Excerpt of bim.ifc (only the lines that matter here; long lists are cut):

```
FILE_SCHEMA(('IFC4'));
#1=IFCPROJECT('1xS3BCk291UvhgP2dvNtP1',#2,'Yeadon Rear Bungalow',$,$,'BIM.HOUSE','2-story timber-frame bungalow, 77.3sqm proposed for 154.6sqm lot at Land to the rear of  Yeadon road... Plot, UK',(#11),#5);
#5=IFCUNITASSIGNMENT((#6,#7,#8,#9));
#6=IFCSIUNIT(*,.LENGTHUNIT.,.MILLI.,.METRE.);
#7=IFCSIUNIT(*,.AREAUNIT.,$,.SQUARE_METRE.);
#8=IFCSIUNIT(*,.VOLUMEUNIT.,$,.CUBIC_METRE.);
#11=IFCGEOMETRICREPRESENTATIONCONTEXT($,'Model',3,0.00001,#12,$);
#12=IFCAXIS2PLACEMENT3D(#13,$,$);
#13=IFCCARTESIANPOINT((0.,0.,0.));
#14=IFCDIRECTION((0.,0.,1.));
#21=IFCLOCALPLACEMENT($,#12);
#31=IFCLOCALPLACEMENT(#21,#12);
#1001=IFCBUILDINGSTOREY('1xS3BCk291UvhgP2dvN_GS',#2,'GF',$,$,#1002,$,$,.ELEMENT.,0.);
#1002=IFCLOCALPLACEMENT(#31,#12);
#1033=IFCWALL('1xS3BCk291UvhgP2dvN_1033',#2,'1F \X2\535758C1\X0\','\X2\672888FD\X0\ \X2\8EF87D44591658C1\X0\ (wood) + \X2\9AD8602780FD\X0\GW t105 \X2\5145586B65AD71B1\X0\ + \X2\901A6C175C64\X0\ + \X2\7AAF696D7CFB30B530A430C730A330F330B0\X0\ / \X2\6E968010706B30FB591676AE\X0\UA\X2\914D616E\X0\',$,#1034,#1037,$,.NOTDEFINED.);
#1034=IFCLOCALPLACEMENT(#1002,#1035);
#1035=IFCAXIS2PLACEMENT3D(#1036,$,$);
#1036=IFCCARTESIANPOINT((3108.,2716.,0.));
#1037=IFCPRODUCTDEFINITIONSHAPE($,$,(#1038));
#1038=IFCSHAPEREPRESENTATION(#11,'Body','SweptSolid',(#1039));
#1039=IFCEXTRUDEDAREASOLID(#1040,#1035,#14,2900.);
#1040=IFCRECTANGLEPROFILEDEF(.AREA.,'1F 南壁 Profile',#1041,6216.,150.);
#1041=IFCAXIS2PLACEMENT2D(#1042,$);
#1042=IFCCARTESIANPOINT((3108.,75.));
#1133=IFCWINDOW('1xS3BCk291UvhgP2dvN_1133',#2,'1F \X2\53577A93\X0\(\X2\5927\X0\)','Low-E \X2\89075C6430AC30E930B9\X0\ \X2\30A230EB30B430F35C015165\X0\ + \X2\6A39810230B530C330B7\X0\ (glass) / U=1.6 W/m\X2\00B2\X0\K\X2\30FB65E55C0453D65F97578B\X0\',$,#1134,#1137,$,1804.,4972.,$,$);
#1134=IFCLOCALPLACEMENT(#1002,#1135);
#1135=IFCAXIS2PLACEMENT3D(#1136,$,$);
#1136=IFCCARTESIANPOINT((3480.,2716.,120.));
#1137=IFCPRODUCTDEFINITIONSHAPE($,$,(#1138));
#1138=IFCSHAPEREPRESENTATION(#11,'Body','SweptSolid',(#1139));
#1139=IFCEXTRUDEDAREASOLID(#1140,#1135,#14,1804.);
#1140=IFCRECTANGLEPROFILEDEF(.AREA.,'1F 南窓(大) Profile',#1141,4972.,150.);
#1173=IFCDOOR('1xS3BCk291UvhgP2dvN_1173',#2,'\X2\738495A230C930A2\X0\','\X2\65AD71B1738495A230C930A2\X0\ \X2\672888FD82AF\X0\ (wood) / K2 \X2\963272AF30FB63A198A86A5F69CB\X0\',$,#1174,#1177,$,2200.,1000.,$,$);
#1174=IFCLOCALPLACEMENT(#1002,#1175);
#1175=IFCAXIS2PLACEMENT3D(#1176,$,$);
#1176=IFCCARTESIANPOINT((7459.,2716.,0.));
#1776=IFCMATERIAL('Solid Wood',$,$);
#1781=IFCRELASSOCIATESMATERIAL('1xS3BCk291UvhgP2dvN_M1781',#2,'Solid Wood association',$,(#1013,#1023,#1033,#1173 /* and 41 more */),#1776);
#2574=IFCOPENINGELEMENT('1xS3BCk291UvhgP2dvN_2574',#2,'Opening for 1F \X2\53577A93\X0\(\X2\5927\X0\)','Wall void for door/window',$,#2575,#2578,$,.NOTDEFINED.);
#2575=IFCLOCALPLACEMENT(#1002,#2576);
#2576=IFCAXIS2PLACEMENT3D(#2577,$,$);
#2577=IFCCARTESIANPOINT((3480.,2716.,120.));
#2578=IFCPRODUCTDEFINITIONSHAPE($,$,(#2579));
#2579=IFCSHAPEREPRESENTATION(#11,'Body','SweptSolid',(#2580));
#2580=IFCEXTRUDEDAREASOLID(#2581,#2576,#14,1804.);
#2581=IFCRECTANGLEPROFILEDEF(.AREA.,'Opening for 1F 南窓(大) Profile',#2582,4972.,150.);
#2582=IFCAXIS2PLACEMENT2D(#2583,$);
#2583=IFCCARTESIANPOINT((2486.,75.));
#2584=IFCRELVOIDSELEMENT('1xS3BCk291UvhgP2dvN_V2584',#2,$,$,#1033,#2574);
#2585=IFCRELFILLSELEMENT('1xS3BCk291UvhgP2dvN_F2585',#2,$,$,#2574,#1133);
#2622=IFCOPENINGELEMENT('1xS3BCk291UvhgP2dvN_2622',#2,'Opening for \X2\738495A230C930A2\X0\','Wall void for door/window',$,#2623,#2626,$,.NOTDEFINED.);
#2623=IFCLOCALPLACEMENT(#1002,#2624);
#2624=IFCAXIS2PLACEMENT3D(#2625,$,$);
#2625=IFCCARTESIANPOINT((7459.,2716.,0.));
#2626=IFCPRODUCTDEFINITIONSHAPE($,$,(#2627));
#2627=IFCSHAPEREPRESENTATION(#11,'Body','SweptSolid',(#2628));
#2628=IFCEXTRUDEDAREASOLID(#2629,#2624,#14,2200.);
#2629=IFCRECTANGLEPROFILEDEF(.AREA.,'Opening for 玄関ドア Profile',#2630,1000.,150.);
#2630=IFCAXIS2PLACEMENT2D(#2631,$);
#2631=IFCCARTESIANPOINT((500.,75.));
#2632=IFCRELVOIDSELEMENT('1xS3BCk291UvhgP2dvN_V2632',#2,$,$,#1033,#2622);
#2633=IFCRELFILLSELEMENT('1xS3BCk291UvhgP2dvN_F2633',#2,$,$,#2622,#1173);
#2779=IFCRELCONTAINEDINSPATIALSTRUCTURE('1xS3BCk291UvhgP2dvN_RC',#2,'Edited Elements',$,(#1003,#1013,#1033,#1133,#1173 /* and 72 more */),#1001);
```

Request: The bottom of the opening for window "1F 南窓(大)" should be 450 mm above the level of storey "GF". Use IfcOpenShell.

```python
import numpy as np
import ifcopenshell
import ifcopenshell.api.geometry
import ifcopenshell.geom
import ifcopenshell.util.element
import ifcopenshell.util.placement
import ifcopenshell.util.shape
import ifcopenshell.util.unit

model = ifcopenshell.open("bim.ifc")
unit_scale = ifcopenshell.util.unit.calculate_unit_scale(model)

window = model.by_guid("1xS3BCk291UvhgP2dvN_1133")
opening = window.FillsVoids[0].RelatingOpeningElement
storey = ifcopenshell.util.element.get_container(window, ifc_class="IfcBuildingStorey")
level = ifcopenshell.util.placement.get_local_placement(storey.ObjectPlacement)[2, 3]

# The opening's origin need not be at the sill, so measure its lowest point.
shape = ifcopenshell.geom.create_shape(ifcopenshell.geom.settings(), opening)
bottom = ifcopenshell.util.shape.get_shape_bottom_elevation(shape, shape.geometry) / unit_scale
dz = level + 0.45 / unit_scale - bottom

shift = np.array([0.0, 0.0, dz])
# The window is not placed relative to its opening, so move both.
for product in (opening, window):
    matrix = ifcopenshell.util.placement.get_local_placement(product.ObjectPlacement)
    matrix[:3, 3] += shift
    ifcopenshell.api.geometry.edit_object_placement(model, product=product, matrix=matrix, is_si=False)

print(f"moved by {dz * unit_scale:+.3f} m")

model.write("bim_updated.ifc")
```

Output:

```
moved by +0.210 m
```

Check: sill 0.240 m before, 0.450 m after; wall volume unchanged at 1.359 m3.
